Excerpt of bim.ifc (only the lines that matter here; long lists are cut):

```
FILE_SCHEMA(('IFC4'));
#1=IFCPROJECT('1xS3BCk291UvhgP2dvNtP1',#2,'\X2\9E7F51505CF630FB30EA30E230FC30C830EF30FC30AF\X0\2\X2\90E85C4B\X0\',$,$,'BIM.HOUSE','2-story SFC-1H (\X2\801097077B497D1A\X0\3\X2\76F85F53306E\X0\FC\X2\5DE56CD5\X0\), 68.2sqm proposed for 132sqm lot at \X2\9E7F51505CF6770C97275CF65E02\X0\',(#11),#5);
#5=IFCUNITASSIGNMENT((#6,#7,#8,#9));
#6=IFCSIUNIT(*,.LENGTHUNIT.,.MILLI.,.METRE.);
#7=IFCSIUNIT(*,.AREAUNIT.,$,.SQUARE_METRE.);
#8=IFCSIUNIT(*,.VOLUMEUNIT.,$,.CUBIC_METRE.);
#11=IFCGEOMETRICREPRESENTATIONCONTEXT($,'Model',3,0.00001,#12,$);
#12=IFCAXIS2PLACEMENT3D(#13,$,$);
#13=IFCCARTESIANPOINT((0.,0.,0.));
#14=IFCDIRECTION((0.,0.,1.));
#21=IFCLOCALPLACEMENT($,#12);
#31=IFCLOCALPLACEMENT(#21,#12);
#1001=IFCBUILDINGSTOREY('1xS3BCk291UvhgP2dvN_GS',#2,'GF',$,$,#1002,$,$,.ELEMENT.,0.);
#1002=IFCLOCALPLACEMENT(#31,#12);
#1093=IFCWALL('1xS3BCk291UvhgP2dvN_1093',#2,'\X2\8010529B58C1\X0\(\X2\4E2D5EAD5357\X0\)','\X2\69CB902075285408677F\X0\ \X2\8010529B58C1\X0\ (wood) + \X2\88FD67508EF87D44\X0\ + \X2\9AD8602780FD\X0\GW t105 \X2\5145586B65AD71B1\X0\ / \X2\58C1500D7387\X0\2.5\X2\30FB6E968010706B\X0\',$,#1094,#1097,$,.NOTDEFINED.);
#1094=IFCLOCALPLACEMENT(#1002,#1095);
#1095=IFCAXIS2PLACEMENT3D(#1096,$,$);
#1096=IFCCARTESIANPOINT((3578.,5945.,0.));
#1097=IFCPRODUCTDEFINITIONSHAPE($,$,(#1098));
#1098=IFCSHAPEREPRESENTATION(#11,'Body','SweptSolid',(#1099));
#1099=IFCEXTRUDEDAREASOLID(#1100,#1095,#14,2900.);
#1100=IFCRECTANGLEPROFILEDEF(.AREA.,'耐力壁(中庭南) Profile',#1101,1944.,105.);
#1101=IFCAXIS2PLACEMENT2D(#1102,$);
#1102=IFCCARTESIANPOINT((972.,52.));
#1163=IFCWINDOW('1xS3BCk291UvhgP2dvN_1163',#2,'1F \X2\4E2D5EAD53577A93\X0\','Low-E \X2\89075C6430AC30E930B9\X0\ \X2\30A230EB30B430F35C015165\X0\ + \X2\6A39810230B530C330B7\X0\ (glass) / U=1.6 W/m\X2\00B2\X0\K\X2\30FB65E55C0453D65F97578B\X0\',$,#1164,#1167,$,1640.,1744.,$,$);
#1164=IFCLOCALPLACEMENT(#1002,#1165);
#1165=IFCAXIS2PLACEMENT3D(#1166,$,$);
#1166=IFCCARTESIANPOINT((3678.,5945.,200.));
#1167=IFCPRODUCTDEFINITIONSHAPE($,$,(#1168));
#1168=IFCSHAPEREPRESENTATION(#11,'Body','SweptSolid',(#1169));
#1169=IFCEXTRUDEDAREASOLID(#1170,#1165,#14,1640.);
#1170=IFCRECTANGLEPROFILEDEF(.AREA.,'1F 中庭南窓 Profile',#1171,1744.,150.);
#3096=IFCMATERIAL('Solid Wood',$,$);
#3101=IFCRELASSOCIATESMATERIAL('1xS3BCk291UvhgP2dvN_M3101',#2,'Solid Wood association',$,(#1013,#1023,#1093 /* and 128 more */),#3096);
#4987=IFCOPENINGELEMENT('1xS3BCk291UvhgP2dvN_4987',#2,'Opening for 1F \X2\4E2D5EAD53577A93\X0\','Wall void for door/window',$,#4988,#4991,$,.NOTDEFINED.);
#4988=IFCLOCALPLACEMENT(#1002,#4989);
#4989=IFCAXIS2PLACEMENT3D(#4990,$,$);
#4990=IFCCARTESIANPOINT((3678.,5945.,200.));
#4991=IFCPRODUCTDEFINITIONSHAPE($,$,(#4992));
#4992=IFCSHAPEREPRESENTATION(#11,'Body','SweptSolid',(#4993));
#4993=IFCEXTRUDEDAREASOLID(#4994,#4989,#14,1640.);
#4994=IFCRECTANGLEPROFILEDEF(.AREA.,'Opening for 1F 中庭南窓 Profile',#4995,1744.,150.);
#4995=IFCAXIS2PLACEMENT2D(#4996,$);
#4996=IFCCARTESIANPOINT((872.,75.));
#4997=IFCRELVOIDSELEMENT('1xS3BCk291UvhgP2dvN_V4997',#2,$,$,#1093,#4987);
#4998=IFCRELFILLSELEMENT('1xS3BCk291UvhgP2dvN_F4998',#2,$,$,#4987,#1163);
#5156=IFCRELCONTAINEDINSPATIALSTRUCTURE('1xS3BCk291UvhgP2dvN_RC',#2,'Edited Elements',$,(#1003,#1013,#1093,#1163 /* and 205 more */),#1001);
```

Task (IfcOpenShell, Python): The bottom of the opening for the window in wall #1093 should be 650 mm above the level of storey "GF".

```python
import numpy as np
import ifcopenshell
import ifcopenshell.api.geometry
import ifcopenshell.geom
import ifcopenshell.util.element
import ifcopenshell.util.placement
import ifcopenshell.util.shape
import ifcopenshell.util.unit

model = ifcopenshell.open("bim.ifc")
unit_scale = ifcopenshell.util.unit.calculate_unit_scale(model)

window = model.by_guid("1xS3BCk291UvhgP2dvN_1163")
opening = window.FillsVoids[0].RelatingOpeningElement
storey = ifcopenshell.util.element.get_container(window, ifc_class="IfcBuildingStorey")
level = ifcopenshell.util.placement.get_local_placement(storey.ObjectPlacement)[2, 3]

# The opening's origin need not be at the sill, so measure its lowest point.
shape = ifcopenshell.geom.create_shape(ifcopenshell.geom.settings(), opening)
bottom = ifcopenshell.util.shape.get_shape_bottom_elevation(shape, shape.geometry) / unit_scale
dz = level + 0.65 / unit_scale - bottom

shift = np.array([0.0, 0.0, dz])
# The window is not placed relative to its opening, so move both.
for product in (opening, window):
    matrix = ifcopenshell.util.placement.get_local_placement(product.ObjectPlacement)
    matrix[:3, 3] += shift
    ifcopenshell.api.geometry.edit_object_placement(model, product=product, matrix=matrix, is_si=False)

print(f"moved by {dz * unit_scale:+.3f} m")

model.write("bim-out.ifc")
```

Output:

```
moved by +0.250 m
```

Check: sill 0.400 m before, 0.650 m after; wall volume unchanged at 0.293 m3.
